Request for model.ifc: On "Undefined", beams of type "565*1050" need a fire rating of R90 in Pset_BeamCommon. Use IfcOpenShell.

First a look at what the model holds.

```python
import ifcopenshell
import ifcopenshell.util.element

model = ifcopenshell.open("model.ifc")
print(model.schema)
storey = next(s for s in model.by_type("IfcBuildingStorey") if s.Name == "Undefined")
beams = [e for e in ifcopenshell.util.element.get_decomposition(storey) if e.is_a("IfcBeam")]
seen = {}
for e in beams:
    element_type = ifcopenshell.util.element.get_type(e)
    key = (element_type.Name if element_type != e and element_type else None, ifcopenshell.util.element.get_pset(e, "Pset_BeamCommon", "FireRating"))
    seen[key] = seen.get(key, 0) + 1
for (name, value), count in sorted(seen.items(), key=str):
    print(count, "x", name, "|", value)
```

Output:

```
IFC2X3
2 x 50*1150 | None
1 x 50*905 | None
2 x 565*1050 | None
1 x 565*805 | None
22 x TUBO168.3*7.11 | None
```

```python
import ifcopenshell
import ifcopenshell.api.pset
import ifcopenshell.util.element

model = ifcopenshell.open("model.ifc")

storey = next(s for s in model.by_type("IfcBuildingStorey") if s.Name == "Undefined")
beams = [e for e in ifcopenshell.util.element.get_decomposition(storey) if e.is_a("IfcBeam")]

count = 0
for e in beams:
    element_type = ifcopenshell.util.element.get_type(e)
    if element_type in (None, e) or element_type.Name != "565*1050":
        continue
    found = ifcopenshell.util.element.get_pset(e, "Pset_BeamCommon", should_inherit=False)
    if found:
        pset = model.by_id(found["id"])
        if len(ifcopenshell.util.element.get_elements_by_pset(pset)) > 1:
            pset = ifcopenshell.api.pset.unshare_pset(model, products=[e], pset=pset)[0]
    else:
        pset = ifcopenshell.api.pset.add_pset(model, product=e, name="Pset_BeamCommon")
    ifcopenshell.api.pset.edit_pset(model, pset=pset, properties={"FireRating": "R90"})
    count += 1

print(count, "beams updated")

model.write("model_rev.ifc")
```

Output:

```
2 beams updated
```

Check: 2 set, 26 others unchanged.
